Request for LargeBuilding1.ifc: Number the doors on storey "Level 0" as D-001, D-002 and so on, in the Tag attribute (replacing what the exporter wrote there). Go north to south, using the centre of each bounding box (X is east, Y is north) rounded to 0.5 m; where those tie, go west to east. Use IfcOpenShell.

First a look at what the model holds.

```python
import ifcopenshell
import ifcopenshell.util.element
import ifcopenshell.util.placement

model = ifcopenshell.open("LargeBuilding1.ifc")
print(model.schema)
storey = next(s for s in model.by_type("IfcBuildingStorey") if s.Name == "Level 0")
doors = [e for e in ifcopenshell.util.element.get_decomposition(storey) if e.is_a("IfcDoor")]
for e in sorted(doors, key=lambda e: e.id()):
    origin = ifcopenshell.util.placement.get_local_placement(e.ObjectPlacement)[:3, 3]
    print(e.id(), e.Tag, e.Name, origin.round(2) + 0.0, sep=" | ")
```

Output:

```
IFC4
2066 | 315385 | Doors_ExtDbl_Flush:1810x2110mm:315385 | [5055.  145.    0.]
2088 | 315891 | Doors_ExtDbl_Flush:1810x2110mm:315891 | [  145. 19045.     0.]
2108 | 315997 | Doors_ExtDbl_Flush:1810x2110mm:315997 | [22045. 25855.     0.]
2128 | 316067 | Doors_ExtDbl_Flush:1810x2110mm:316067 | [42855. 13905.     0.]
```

```python
import ifcopenshell
import ifcopenshell.geom
import ifcopenshell.util.element
import ifcopenshell.util.shape

model = ifcopenshell.open("LargeBuilding1.ifc")
settings = ifcopenshell.geom.settings()
settings.set("use-world-coords", True)


def centre(element):
    shape = ifcopenshell.geom.create_shape(settings, element)
    return ifcopenshell.util.shape.get_bbox_centroid(shape.geometry)


storey = next(s for s in model.by_type("IfcBuildingStorey") if s.Name == "Level 0")
doors = [e for e in ifcopenshell.util.element.get_decomposition(storey) if e.is_a("IfcDoor")]

# Insertion points can sit at a corner or the storey origin, so sort by the geometry (in metres).
centres = {e: centre(e) for e in doors}
doors.sort(key=lambda e: (-round(centres[e][1] / 0.5), centres[e][0]))

for i, e in enumerate(doors, start=1):
    number = f"D-0{i:02d}"
    e.Tag = number
    print(e.id(), number)

model.write("LargeBuilding1_rev.ifc")
```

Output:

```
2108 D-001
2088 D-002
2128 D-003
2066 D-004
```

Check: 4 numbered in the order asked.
